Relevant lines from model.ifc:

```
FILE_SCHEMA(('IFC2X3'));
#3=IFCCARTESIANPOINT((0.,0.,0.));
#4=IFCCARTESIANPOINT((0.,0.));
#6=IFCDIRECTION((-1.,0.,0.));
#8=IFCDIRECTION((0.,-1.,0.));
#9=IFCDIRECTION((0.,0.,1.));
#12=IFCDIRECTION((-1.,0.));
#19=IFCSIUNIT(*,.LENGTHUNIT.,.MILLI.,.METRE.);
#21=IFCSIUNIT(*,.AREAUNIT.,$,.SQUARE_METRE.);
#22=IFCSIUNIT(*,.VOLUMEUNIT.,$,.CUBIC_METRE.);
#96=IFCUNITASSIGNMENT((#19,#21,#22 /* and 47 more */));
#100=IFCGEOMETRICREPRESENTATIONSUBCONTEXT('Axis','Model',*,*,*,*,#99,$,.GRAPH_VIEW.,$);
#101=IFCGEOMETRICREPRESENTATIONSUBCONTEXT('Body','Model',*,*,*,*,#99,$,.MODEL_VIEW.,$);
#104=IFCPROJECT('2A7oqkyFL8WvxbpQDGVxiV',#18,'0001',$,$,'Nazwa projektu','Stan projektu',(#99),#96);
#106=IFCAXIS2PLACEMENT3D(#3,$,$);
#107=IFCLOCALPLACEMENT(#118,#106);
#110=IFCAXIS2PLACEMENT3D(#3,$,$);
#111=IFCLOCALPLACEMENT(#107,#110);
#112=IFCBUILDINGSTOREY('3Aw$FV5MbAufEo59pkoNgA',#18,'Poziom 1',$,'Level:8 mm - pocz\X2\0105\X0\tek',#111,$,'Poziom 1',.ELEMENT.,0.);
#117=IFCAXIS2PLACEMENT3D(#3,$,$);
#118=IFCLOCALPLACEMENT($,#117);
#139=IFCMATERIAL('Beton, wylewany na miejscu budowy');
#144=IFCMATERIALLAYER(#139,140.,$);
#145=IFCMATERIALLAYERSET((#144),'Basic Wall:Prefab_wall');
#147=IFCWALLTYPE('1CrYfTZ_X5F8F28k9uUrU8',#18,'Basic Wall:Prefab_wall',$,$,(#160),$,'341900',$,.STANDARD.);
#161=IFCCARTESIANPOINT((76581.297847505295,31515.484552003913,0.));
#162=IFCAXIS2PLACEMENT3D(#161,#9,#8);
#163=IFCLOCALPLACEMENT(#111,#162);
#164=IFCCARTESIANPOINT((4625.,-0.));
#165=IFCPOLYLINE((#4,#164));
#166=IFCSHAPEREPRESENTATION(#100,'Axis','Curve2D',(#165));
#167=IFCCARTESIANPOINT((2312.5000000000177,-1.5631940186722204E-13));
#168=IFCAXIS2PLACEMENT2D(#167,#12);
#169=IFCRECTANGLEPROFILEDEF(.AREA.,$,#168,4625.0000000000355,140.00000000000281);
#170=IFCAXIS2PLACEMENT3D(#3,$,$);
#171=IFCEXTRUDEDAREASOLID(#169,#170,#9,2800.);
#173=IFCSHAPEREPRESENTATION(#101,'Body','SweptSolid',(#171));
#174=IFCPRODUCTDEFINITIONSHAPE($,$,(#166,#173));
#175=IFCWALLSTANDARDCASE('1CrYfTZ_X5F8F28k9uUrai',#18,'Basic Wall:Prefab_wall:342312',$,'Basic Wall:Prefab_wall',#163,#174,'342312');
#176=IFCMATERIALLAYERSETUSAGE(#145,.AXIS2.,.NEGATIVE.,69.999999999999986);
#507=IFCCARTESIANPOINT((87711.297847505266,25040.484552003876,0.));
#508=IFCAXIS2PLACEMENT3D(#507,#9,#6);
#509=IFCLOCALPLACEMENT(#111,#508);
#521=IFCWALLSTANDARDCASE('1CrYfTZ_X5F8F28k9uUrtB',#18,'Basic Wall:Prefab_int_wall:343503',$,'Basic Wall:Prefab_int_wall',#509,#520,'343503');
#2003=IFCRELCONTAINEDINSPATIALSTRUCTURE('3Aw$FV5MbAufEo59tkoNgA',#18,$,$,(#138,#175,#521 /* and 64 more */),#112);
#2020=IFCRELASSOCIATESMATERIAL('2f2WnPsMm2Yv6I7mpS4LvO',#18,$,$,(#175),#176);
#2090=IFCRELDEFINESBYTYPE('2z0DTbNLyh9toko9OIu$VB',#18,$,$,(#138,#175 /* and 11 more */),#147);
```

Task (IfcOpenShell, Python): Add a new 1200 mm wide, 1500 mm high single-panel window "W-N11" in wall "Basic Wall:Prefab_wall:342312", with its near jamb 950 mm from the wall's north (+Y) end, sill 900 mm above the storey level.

```python
import numpy as np
import ifcopenshell
import ifcopenshell.api.feature
import ifcopenshell.api.geometry
import ifcopenshell.api.root
import ifcopenshell.api.spatial
import ifcopenshell.api.type
import ifcopenshell.geom
import ifcopenshell.util.element
import ifcopenshell.util.placement
import ifcopenshell.util.representation
import ifcopenshell.util.shape
import ifcopenshell.util.unit

model = ifcopenshell.open("model.ifc")
unit_scale = ifcopenshell.util.unit.calculate_unit_scale(model)
settings = ifcopenshell.geom.settings()


def volume(element):
    """Net volume in cubic metres, openings subtracted."""
    shape = ifcopenshell.geom.create_shape(settings, element)
    return ifcopenshell.util.shape.get_volume(shape.geometry)


wall = model.by_guid("1CrYfTZ_X5F8F28k9uUrai")
storey = ifcopenshell.util.element.get_container(wall, ifc_class="IfcBuildingStorey")
context = ifcopenshell.util.representation.get_context(model, "Model", "Body", "MODEL_VIEW")
before = volume(wall)

width, height, from_end, sill = 1.2, 1.5, 0.95, 0.9  # metres

# The wall runs along its own X axis, and the end named is its -X end.
wall_shape = ifcopenshell.geom.create_shape(settings, wall)
x, y, z = ifcopenshell.util.shape.get_vertices(wall_shape.geometry).T
start = x.min() + from_end
face, thickness = float(y.min()), float(y.max() - y.min())
wall_matrix = ifcopenshell.util.placement.get_local_placement(wall.ObjectPlacement)
level = ifcopenshell.util.placement.get_local_placement(storey.ObjectPlacement)[2, 3]


def in_wall(x, y):
    """Placement at x, y metres in the wall's axes, at sill height."""
    matrix = wall_matrix.copy()
    matrix[:, 3] = wall_matrix @ np.array([x / unit_scale, y / unit_scale, 0.0, 1.0])
    matrix[2, 3] = level + sill / unit_scale
    return matrix


# Opening: a box that overshoots both wall faces by 50 mm.
opening = ifcopenshell.api.root.create_entity(model, ifc_class="IfcOpeningElement")
box = ifcopenshell.api.geometry.add_wall_representation(
    model, context=context, length=width, height=height, thickness=thickness + 0.1
)
ifcopenshell.api.geometry.assign_representation(model, product=opening, representation=box)
ifcopenshell.api.geometry.edit_object_placement(model, product=opening, matrix=in_wall(start, face - 0.05), is_si=False)
ifcopenshell.api.feature.add_feature(model, feature=opening, element=wall)

window = ifcopenshell.api.root.create_entity(model, ifc_class="IfcWindow", name="W-N11")
window.OverallWidth, window.OverallHeight = width / unit_scale, height / unit_scale
body = ifcopenshell.api.geometry.add_window_representation(
    model,
    context=context,
    overall_width=window.OverallWidth,
    overall_height=window.OverallHeight,
    partition_type="SINGLE_PANEL",
)
ifcopenshell.api.geometry.assign_representation(model, product=window, representation=body)
ifcopenshell.api.spatial.assign_container(model, products=[window], relating_structure=storey)
fills = ifcopenshell.api.feature.add_filling(model, opening=opening, element=window)
fills.OwnerHistory = window.OwnerHistory  # required in IFC2X3

# IFC2X3 keeps the operation on the window style.
style = ifcopenshell.api.root.create_entity(model, ifc_class="IfcWindowStyle", name="W-N11")
style.OperationType, style.ConstructionType = "SINGLE_PANEL", "NOTDEFINED"
style.ParameterTakesPrecedence = style.Sizeable = False
ifcopenshell.api.type.assign_type(model, related_objects=[window], relating_type=style)

# Centre the window in the wall's thickness.
ifcopenshell.api.geometry.edit_object_placement(model, product=window, matrix=in_wall(start, face), is_si=False)
window_shape = ifcopenshell.geom.create_shape(settings, window)
depth = ifcopenshell.util.shape.get_vertices(window_shape.geometry)[:, 1]
offset = face + thickness / 2 - (depth.min() + depth.max()) / 2
ifcopenshell.api.geometry.edit_object_placement(model, product=window, matrix=in_wall(start, offset), is_si=False)

after = volume(wall)

print(f"wall volume {before:.3f} -> {after:.3f} m3")

model.write("model_rev.ifc")
```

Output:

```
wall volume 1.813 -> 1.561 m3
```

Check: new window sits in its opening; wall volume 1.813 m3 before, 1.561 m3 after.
